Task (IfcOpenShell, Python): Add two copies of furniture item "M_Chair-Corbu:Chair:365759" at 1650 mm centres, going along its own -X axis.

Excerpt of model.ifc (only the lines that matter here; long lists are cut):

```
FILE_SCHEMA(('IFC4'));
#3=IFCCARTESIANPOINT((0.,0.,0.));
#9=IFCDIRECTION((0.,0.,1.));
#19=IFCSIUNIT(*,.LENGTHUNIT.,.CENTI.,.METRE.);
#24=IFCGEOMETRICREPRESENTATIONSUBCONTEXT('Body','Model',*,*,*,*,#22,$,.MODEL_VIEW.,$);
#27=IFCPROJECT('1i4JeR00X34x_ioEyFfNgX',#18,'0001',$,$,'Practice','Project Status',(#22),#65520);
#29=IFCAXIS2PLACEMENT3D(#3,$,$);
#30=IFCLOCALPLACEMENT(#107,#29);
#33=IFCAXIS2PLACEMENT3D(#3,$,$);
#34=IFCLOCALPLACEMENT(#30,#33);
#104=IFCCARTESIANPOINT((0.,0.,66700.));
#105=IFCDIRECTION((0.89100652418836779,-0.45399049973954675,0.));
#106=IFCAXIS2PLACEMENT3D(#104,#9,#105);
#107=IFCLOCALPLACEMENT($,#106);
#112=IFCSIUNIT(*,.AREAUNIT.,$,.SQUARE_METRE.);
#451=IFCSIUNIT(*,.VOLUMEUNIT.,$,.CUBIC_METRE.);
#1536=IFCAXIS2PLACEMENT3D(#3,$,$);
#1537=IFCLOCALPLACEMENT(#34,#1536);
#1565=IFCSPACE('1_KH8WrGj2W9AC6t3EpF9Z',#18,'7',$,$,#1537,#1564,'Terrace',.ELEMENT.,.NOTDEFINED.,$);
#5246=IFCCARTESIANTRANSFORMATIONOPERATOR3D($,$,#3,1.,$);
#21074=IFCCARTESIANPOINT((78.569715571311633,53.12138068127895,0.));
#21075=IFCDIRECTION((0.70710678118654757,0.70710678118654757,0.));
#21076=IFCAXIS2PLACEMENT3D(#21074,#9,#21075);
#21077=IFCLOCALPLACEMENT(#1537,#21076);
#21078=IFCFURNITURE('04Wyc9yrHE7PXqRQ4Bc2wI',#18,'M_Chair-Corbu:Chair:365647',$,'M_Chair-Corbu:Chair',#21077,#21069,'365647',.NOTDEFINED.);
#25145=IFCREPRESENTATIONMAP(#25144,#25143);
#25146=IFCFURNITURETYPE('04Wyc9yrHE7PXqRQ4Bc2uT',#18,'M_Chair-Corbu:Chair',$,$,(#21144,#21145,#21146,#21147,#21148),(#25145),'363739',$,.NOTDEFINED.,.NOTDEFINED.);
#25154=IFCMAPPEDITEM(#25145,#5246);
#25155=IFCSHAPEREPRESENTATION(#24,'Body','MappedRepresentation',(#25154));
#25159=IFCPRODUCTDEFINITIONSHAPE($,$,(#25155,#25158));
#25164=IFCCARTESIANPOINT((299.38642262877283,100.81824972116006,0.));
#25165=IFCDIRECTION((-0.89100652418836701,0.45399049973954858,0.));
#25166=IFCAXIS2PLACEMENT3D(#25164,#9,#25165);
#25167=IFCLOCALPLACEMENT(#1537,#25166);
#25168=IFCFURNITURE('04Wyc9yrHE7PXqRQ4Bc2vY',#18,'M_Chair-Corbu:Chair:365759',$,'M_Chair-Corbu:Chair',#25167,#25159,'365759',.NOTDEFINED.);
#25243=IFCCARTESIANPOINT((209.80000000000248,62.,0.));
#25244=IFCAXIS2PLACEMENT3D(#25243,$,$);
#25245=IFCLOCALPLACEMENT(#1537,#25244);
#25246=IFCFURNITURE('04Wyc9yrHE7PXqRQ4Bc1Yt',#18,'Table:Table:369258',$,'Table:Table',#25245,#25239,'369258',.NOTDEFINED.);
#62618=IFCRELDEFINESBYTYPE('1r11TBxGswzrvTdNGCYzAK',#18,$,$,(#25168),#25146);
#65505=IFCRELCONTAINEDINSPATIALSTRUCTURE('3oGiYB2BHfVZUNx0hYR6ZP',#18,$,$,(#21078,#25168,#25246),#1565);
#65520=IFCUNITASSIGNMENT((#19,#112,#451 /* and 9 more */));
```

```python
import ifcopenshell
import ifcopenshell.api.geometry
import ifcopenshell.api.root
import ifcopenshell.util.element
import ifcopenshell.util.placement
import ifcopenshell.util.unit

model = ifcopenshell.open("model.ifc")
unit_scale = ifcopenshell.util.unit.calculate_unit_scale(model)


def reuse_history(source, copy):
    """copy_class also copies each property set's owner history, people and application; keep the originals."""
    for rel in copy.IsDefinedBy:
        if rel.is_a("IfcRelDefinesByProperties") and (history := rel.RelatingPropertyDefinition.OwnerHistory):
            rel.RelatingPropertyDefinition.OwnerHistory = source.OwnerHistory
            ifcopenshell.util.element.remove_deep2(model, history)


source = model.by_id(25168)
base = ifcopenshell.util.placement.get_local_placement(source.ObjectPlacement)
step = -base[:3, 0] * 1.65 / unit_scale

for i in range(1, 3):
    copy = ifcopenshell.api.root.copy_class(model, product=source)
    copy.Representation = ifcopenshell.util.element.copy_deep(
        model, source.Representation, exclude=["IfcGeometricRepresentationContext", "IfcRepresentationMap"]
    )
    copy.Name = "M_Chair-Corbu:Chair"
    copy.Tag = None
    reuse_history(source, copy)
    matrix = base.copy()
    matrix[:3, 3] += i * step
    print("added at", matrix[:3, 3].round(3) + 0.0)
    ifcopenshell.api.geometry.edit_object_placement(model, product=copy, matrix=matrix, is_si=False)

model.write("model-out.ifc")
```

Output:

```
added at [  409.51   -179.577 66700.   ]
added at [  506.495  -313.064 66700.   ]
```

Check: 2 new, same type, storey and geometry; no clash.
